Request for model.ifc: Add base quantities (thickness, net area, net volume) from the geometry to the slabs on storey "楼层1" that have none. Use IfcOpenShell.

First a look at what the model holds.

```python
import ifcopenshell
import ifcopenshell.util.element
import ifcopenshell.util.unit

model = ifcopenshell.open("model.ifc")
print(model.schema)
for unit_type in ("LENGTHUNIT", "AREAUNIT", "VOLUMEUNIT"):
    print(unit_type, ifcopenshell.util.unit.calculate_unit_scale(model, unit_type))
storey = next(s for s in model.by_type("IfcBuildingStorey") if s.Name == "楼层1")
slabs = [e for e in ifcopenshell.util.element.get_decomposition(storey) if e.is_a("IfcSlab")]
for e in sorted(slabs, key=lambda e: e.id()):
    print(e.id(), e.is_a(), e.Name, list(ifcopenshell.util.element.get_psets(e, qtos_only=True)), sep=" | ")
```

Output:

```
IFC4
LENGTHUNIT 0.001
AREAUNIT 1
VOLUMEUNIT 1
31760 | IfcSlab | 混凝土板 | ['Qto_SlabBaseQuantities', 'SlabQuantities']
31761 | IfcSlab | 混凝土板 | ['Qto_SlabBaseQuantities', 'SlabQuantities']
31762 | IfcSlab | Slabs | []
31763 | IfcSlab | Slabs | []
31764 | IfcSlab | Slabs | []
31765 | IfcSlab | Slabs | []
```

```python
import ifcopenshell
import ifcopenshell.api.pset
import ifcopenshell.geom
import ifcopenshell.util.element
import ifcopenshell.util.shape
import ifcopenshell.util.unit

model = ifcopenshell.open("model.ifc")
unit_scale = ifcopenshell.util.unit.calculate_unit_scale(model)
area_scale = ifcopenshell.util.unit.calculate_unit_scale(model, "AREAUNIT")
volume_scale = ifcopenshell.util.unit.calculate_unit_scale(model, "VOLUMEUNIT")
settings = ifcopenshell.geom.settings()

storey = next(s for s in model.by_type("IfcBuildingStorey") if s.Name == "楼层1")
slabs = [e for e in ifcopenshell.util.element.get_decomposition(storey) if e.is_a("IfcSlab")]

for e in sorted(slabs, key=lambda e: e.id()):
    if ifcopenshell.util.element.get_psets(e, qtos_only=True, should_inherit=False):
        continue
    # Geometry comes back in metres, in the element's own axes.
    shape = ifcopenshell.geom.create_shape(settings, e)
    values = {
        "Width": ifcopenshell.util.shape.get_z(shape.geometry) / unit_scale,
        "NetArea": ifcopenshell.util.shape.get_footprint_area(shape.geometry) / area_scale,
        "NetVolume": ifcopenshell.util.shape.get_volume(shape.geometry) / volume_scale,
    }
    qto = ifcopenshell.api.pset.add_qto(model, product=e, name="Qto_SlabBaseQuantities")
    ifcopenshell.api.pset.edit_qto(model, qto=qto, properties=values)
    print(e.id(), {k: round(v, 3) for k, v in values.items()})

model.write("model_v2.ifc")
```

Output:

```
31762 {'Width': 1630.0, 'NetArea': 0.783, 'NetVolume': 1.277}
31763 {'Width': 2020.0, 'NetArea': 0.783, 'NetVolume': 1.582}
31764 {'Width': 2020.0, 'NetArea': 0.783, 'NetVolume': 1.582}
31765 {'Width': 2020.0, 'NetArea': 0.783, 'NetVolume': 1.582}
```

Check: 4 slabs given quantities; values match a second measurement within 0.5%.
